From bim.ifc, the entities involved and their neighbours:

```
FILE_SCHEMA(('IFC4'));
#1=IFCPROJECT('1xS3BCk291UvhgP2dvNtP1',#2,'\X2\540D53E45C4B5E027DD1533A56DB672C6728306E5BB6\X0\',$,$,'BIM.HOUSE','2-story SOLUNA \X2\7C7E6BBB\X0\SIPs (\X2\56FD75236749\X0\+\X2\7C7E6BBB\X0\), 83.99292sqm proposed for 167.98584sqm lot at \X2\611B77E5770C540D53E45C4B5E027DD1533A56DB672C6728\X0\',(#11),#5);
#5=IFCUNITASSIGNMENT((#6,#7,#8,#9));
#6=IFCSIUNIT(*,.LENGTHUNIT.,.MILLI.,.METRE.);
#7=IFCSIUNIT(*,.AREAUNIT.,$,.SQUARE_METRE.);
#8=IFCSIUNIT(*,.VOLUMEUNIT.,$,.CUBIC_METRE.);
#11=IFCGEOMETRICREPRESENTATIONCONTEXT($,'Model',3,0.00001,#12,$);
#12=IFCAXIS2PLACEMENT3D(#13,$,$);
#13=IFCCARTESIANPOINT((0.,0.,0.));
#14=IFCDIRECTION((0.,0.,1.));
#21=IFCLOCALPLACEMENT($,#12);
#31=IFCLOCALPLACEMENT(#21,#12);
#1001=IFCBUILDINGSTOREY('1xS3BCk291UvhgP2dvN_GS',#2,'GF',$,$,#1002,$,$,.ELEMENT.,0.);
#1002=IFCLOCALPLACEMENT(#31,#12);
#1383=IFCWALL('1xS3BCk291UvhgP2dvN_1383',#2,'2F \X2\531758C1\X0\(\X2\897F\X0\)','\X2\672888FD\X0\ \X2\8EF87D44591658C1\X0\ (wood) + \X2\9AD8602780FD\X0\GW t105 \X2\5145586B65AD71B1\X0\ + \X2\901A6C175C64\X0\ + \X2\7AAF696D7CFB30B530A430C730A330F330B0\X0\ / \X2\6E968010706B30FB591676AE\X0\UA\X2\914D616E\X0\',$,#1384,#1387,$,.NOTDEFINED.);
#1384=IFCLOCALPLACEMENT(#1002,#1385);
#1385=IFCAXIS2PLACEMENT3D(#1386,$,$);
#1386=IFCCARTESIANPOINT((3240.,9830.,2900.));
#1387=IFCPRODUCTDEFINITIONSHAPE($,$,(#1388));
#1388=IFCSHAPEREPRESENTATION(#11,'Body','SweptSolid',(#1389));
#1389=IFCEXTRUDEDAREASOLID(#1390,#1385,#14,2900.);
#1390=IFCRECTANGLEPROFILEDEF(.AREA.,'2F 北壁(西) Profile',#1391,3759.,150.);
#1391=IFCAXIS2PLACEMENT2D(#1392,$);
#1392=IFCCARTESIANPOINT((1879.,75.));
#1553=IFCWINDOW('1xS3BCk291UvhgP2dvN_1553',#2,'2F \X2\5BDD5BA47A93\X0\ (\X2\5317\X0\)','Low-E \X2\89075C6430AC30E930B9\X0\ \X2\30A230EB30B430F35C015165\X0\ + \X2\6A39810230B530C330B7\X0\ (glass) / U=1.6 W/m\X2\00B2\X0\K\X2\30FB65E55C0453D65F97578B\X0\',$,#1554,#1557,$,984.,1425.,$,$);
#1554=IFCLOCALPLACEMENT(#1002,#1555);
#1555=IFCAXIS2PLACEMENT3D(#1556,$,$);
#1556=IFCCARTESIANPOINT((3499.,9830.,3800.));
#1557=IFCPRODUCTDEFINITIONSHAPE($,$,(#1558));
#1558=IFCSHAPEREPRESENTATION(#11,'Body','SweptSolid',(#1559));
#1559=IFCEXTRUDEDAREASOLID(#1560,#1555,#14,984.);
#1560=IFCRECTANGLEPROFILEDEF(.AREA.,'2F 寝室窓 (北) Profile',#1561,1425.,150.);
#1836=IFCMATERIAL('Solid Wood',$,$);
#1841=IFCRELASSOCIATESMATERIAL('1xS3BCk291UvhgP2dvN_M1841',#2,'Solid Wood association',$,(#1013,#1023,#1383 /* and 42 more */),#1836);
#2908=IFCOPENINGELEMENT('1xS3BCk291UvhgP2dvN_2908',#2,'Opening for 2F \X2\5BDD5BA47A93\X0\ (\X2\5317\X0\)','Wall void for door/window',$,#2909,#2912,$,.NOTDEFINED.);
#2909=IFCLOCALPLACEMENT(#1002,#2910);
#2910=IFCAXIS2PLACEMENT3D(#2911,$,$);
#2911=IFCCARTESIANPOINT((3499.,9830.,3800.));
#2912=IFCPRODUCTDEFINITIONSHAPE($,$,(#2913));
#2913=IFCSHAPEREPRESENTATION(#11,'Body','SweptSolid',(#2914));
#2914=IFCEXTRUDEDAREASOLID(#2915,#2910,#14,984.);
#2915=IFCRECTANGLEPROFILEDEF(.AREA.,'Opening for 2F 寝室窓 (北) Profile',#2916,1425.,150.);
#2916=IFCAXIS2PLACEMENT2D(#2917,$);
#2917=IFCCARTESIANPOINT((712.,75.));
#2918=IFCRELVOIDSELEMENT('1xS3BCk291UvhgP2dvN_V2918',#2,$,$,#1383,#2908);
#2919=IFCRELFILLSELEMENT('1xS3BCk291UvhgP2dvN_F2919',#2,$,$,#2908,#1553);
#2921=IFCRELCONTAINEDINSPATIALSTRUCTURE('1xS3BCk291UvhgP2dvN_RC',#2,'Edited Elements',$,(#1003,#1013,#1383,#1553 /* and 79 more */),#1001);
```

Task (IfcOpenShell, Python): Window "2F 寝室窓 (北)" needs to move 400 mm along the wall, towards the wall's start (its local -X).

```python
import ifcopenshell
import ifcopenshell.api.geometry
import ifcopenshell.util.placement

model = ifcopenshell.open("bim.ifc")

window = model.by_guid("1xS3BCk291UvhgP2dvN_1553")
opening = window.FillsVoids[0].RelatingOpeningElement
wall = opening.VoidsElements[0].RelatingBuildingElement

wall_matrix = ifcopenshell.util.placement.get_local_placement(wall.ObjectPlacement)
shift = wall_matrix[:3, 0] * -400.0
before = ifcopenshell.util.placement.get_local_placement(window.ObjectPlacement)[:3, 3].copy()

# The window is not placed relative to its opening, so move both.
for product in (opening, window):
    matrix = ifcopenshell.util.placement.get_local_placement(product.ObjectPlacement)
    matrix[:3, 3] += shift
    ifcopenshell.api.geometry.edit_object_placement(model, product=product, matrix=matrix, is_si=False)

after = ifcopenshell.util.placement.get_local_placement(window.ObjectPlacement)[:3, 3]
print("window moved by", (after - before).round(3) + 0.0)

model.write("bim_v2.ifc")
```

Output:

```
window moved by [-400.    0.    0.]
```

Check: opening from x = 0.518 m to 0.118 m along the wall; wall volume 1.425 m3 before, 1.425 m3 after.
